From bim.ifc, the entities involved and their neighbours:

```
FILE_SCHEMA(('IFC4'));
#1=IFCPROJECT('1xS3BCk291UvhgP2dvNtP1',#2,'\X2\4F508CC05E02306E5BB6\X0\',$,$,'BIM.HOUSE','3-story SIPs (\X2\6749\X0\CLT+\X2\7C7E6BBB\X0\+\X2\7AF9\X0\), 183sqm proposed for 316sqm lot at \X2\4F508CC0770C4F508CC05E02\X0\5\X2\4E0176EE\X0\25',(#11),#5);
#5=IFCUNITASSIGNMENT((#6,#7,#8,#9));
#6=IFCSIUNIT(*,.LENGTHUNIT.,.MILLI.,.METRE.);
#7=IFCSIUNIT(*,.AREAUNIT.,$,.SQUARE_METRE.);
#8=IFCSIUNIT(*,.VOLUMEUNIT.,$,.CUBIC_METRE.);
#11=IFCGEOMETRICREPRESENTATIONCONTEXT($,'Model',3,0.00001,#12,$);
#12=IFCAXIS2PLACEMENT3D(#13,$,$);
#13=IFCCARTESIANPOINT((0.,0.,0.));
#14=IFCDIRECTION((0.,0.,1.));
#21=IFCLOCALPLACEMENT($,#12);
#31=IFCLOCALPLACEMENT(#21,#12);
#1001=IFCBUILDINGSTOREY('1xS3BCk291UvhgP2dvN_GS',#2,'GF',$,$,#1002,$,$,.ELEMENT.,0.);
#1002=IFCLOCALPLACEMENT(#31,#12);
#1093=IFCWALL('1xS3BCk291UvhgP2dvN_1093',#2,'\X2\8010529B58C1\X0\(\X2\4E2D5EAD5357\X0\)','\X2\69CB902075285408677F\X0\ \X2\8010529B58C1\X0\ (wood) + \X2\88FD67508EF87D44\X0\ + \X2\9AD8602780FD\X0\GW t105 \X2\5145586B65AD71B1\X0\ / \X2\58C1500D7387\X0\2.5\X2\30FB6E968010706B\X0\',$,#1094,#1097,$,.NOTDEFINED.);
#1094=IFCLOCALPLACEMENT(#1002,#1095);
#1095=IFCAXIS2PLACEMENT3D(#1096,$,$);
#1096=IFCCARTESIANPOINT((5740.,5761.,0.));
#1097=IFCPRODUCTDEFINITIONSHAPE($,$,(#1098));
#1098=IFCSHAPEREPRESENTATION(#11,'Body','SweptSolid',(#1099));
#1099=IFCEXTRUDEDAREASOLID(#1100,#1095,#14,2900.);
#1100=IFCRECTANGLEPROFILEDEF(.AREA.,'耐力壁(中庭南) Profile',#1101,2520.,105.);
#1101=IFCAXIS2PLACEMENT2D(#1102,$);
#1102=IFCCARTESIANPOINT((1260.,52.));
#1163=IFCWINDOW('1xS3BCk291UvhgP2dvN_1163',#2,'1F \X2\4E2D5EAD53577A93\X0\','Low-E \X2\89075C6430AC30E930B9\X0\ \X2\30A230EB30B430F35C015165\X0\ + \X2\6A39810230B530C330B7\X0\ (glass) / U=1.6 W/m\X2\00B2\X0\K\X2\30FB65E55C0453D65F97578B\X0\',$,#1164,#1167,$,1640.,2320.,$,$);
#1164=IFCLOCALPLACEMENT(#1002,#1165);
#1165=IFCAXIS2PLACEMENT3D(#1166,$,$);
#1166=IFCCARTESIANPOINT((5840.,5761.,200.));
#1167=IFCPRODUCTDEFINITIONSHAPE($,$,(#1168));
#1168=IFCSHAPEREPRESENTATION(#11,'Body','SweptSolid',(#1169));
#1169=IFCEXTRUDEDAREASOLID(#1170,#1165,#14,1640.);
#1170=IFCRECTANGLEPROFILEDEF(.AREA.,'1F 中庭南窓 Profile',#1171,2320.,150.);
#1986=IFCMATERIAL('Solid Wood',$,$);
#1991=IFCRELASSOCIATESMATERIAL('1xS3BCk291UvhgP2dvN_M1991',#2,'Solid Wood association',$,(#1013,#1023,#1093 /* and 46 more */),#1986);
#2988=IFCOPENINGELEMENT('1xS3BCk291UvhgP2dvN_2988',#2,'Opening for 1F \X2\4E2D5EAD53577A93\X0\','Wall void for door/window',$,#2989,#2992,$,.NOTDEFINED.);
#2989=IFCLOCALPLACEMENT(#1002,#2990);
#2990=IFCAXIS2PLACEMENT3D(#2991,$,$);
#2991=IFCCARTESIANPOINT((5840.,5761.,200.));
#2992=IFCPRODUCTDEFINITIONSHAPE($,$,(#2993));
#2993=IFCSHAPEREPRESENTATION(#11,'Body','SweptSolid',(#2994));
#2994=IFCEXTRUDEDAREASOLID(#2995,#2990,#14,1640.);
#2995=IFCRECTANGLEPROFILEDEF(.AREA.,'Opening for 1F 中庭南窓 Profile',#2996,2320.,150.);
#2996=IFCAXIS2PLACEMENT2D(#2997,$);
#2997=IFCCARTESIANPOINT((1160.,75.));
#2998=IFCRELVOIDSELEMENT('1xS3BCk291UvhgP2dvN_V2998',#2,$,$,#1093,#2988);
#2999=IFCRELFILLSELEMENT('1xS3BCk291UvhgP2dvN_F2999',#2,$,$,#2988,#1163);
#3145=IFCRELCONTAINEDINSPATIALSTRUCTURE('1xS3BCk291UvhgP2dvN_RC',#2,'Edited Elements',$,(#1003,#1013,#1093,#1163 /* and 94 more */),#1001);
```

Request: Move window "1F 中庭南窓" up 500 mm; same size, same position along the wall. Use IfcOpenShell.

```python
import numpy as np
import ifcopenshell
import ifcopenshell.api.geometry
import ifcopenshell.util.placement
import ifcopenshell.util.unit

model = ifcopenshell.open("bim.ifc")
unit_scale = ifcopenshell.util.unit.calculate_unit_scale(model)

window = model.by_guid("1xS3BCk291UvhgP2dvN_1163")
opening = window.FillsVoids[0].RelatingOpeningElement
dz = 0.5 / unit_scale

shift = np.array([0.0, 0.0, dz])
# The window is not placed relative to its opening, so move both.
for product in (opening, window):
    matrix = ifcopenshell.util.placement.get_local_placement(product.ObjectPlacement)
    matrix[:3, 3] += shift
    ifcopenshell.api.geometry.edit_object_placement(model, product=product, matrix=matrix, is_si=False)

print(f"moved by {dz * unit_scale:+.3f} m")

model.write("bim_edited.ifc")
```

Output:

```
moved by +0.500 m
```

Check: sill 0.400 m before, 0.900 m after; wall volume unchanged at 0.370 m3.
